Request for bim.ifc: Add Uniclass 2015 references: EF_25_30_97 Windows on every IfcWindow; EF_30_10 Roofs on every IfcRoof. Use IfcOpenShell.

First a look at what the model holds.

```python
import ifcopenshell

model = ifcopenshell.open("bim.ifc")
print(model.schema)
print("classifications:", [c.Name for c in model.by_type("IfcClassification")])
for ifc_class in ("IfcDoor", "IfcRoof", "IfcStair", "IfcWall", "IfcWindow"):
    print(ifc_class, len(model.by_type(ifc_class)))
```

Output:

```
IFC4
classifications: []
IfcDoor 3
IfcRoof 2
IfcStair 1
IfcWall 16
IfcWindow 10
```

```python
import ifcopenshell
import ifcopenshell.api.classification

model = ifcopenshell.open("bim.ifc")

system = ifcopenshell.api.classification.add_classification(model, classification="Uniclass 2015")

codes = {
    "IfcWindow": ("EF_25_30_97", "Windows"),
    "IfcRoof": ("EF_30_10", "Roofs"),
}
for ifc_class, (code, name) in codes.items():
    products = model.by_type(ifc_class)
    ifcopenshell.api.classification.add_reference(
        model, products=products, classification=system, identification=code, name=name
    )
    print(code, len(products))

model.write("bim_updated.ifc")
```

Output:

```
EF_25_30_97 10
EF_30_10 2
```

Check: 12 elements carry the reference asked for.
